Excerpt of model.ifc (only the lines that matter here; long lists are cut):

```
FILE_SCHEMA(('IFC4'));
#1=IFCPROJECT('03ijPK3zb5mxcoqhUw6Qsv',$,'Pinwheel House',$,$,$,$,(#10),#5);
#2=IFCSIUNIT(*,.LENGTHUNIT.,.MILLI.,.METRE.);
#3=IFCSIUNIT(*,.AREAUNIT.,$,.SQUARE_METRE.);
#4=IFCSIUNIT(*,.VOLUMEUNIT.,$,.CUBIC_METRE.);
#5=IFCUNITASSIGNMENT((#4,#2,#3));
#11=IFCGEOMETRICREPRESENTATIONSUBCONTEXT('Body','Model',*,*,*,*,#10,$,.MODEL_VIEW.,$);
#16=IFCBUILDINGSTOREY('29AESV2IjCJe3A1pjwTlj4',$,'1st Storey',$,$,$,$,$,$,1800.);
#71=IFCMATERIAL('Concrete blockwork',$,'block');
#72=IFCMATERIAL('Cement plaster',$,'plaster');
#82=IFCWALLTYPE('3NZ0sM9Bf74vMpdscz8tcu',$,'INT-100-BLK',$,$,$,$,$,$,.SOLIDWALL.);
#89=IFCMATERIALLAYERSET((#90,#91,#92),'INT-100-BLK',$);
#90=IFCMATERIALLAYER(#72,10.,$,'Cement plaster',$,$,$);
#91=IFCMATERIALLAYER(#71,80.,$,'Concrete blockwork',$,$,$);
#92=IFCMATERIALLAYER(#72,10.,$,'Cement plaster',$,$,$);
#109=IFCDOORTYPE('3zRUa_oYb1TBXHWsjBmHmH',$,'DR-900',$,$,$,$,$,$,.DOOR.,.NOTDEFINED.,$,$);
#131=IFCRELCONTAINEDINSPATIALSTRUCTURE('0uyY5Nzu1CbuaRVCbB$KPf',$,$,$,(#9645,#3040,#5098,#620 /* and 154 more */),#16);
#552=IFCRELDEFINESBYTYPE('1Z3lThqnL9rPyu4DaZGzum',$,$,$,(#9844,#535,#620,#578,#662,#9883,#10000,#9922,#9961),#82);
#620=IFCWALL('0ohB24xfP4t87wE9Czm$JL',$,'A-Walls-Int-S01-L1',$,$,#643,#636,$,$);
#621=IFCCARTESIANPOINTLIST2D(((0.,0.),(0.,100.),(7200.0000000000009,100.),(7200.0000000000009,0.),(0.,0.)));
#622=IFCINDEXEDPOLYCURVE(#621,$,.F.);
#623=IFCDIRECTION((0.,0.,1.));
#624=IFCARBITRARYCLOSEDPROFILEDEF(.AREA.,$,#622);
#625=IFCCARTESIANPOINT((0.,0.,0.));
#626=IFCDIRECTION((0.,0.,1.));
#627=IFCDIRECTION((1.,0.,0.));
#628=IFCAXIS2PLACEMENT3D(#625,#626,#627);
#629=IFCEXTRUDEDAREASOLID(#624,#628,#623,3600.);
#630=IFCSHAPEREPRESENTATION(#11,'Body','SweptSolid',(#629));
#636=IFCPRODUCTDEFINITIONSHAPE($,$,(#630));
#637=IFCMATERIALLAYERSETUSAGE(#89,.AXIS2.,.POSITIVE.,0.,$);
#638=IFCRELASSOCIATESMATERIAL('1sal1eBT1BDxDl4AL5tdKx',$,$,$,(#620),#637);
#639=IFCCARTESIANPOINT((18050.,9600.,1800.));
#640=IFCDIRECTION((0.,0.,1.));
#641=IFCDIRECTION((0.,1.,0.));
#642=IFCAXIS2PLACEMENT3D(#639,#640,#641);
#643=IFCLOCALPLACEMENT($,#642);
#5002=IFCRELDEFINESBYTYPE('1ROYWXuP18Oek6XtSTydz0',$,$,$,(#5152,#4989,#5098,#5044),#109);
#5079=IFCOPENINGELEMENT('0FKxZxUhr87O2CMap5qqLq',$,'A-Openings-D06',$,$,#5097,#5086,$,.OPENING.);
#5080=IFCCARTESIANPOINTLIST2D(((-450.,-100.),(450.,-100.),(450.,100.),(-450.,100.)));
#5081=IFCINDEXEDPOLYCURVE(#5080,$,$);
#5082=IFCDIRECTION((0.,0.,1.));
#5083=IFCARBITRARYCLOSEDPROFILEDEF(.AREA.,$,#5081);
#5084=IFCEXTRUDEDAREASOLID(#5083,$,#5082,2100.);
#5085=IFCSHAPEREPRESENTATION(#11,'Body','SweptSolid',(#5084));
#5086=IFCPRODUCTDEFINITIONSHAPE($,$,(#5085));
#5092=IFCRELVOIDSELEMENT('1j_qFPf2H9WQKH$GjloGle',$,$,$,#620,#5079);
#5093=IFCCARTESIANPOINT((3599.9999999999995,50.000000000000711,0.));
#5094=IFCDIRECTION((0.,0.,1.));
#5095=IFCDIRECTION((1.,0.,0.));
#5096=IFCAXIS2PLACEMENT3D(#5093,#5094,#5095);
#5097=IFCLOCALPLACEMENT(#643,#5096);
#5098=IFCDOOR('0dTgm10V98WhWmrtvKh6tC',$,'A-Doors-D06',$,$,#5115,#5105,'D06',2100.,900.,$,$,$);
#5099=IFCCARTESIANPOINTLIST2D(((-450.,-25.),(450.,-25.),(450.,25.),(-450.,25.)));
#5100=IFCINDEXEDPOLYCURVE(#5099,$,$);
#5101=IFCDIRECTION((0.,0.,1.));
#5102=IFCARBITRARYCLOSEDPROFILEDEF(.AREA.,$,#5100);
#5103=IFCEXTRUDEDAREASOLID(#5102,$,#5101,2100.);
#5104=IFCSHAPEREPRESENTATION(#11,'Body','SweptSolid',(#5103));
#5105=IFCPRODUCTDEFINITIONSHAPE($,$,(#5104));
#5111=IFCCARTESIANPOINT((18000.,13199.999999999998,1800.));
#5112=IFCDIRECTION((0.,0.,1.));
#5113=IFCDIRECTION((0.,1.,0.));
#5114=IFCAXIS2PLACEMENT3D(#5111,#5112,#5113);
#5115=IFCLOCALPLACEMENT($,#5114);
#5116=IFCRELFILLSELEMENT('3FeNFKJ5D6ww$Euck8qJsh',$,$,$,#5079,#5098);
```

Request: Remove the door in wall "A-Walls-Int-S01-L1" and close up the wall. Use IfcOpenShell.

```python
import ifcopenshell
import ifcopenshell.api.feature
import ifcopenshell.api.root
import ifcopenshell.geom
import ifcopenshell.util.shape

model = ifcopenshell.open("model.ifc")
settings = ifcopenshell.geom.settings()


def volume(element):
    """Net volume in cubic metres, openings subtracted."""
    shape = ifcopenshell.geom.create_shape(settings, element)
    return ifcopenshell.util.shape.get_volume(shape.geometry)


door = model.by_guid("0dTgm10V98WhWmrtvKh6tC")
opening = door.FillsVoids[0].RelatingOpeningElement
wall = opening.VoidsElements[0].RelatingBuildingElement
before = volume(wall)

ifcopenshell.api.root.remove_product(model, product=door)
ifcopenshell.api.feature.remove_feature(model, feature=opening)

after = volume(wall)

print(f"wall volume {before:.3f} -> {after:.3f} m3")

model.write("model_v2.ifc")
```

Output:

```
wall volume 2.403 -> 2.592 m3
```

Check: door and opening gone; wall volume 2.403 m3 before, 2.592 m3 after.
